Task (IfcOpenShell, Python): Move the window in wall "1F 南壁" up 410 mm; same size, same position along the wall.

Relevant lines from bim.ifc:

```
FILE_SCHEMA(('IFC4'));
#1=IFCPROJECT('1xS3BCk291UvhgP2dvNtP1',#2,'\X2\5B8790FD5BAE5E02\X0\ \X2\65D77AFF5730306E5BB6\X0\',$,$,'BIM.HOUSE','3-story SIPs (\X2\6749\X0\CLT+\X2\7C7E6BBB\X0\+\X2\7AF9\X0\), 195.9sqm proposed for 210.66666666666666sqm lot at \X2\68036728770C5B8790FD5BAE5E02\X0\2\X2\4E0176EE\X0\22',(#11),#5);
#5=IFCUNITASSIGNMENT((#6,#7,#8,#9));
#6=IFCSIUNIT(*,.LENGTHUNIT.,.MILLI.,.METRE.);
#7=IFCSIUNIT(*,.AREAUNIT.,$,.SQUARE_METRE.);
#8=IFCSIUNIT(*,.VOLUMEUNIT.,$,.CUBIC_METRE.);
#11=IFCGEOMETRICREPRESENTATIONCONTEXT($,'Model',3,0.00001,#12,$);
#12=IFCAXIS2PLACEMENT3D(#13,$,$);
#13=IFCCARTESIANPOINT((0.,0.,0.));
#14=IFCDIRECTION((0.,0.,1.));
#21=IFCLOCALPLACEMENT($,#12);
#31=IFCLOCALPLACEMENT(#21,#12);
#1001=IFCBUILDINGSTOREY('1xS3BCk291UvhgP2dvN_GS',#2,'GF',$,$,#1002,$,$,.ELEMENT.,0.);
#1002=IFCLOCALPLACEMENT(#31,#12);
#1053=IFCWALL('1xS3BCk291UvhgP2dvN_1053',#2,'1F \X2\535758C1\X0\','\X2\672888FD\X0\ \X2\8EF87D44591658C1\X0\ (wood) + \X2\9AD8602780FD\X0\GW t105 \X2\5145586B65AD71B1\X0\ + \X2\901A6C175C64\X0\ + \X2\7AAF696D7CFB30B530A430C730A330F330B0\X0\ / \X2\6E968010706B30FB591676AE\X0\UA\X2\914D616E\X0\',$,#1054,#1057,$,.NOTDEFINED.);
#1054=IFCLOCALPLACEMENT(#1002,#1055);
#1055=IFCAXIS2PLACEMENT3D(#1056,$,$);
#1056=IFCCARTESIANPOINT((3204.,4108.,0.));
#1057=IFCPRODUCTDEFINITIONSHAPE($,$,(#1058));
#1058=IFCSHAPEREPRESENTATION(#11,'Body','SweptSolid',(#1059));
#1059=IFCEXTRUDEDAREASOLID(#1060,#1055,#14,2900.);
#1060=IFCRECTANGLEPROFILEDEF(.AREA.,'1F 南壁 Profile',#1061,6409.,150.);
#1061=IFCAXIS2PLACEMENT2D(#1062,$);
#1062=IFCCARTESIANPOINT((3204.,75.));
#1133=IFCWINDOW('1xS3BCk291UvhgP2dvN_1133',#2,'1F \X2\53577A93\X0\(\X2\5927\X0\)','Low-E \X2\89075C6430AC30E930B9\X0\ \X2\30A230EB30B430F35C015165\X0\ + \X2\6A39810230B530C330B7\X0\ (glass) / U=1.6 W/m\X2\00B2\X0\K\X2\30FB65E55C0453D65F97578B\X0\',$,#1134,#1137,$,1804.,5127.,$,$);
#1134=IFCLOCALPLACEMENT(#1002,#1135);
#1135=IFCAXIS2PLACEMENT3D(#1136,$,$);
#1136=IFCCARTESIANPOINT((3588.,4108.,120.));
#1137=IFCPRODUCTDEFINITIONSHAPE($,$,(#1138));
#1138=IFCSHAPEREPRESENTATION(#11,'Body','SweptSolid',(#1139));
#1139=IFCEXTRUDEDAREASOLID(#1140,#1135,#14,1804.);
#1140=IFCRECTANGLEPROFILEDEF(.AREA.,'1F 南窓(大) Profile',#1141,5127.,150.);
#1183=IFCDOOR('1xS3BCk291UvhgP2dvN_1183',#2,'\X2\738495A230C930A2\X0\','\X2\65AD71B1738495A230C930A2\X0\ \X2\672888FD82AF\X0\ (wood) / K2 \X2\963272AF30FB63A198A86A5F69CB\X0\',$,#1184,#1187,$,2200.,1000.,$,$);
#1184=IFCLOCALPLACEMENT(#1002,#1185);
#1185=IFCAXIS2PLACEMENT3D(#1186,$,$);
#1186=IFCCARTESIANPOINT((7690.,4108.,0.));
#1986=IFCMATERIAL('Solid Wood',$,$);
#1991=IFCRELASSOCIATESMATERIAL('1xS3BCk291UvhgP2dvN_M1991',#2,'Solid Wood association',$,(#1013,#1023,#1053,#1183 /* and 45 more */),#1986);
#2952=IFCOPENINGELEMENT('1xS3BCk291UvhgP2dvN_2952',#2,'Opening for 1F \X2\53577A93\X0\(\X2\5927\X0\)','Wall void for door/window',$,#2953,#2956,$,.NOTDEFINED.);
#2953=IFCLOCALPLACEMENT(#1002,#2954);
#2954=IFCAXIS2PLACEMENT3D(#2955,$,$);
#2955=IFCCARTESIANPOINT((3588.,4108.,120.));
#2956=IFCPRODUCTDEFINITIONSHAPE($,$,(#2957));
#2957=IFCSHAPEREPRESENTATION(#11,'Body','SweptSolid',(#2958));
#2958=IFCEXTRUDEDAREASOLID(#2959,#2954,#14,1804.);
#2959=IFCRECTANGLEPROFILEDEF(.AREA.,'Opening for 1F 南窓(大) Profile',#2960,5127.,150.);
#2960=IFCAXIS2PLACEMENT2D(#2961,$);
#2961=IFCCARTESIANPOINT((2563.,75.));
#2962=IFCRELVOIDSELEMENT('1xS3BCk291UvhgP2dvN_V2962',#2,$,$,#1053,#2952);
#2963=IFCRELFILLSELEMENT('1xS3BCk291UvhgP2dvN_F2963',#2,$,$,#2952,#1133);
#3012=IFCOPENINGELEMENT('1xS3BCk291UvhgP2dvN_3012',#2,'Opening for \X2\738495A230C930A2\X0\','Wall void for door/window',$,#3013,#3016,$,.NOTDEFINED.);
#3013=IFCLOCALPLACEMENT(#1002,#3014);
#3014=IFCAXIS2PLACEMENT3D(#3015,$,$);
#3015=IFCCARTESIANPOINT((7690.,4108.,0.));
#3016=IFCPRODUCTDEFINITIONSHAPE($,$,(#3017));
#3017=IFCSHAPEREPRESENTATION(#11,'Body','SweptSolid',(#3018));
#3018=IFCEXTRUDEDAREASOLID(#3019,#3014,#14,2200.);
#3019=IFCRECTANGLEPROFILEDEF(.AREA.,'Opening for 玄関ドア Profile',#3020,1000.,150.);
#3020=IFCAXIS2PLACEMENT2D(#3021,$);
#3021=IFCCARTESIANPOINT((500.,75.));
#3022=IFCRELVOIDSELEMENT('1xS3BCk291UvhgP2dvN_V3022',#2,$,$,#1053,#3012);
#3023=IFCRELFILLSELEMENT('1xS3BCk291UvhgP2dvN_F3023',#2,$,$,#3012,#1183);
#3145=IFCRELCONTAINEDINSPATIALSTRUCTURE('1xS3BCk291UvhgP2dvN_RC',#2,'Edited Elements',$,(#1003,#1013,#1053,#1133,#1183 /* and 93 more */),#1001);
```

```python
import numpy as np
import ifcopenshell
import ifcopenshell.api.geometry
import ifcopenshell.util.placement
import ifcopenshell.util.unit

model = ifcopenshell.open("bim.ifc")
unit_scale = ifcopenshell.util.unit.calculate_unit_scale(model)

window = model.by_guid("1xS3BCk291UvhgP2dvN_1133")
opening = window.FillsVoids[0].RelatingOpeningElement
dz = 0.41 / unit_scale

shift = np.array([0.0, 0.0, dz])
# The window is not placed relative to its opening, so move both.
for product in (opening, window):
    matrix = ifcopenshell.util.placement.get_local_placement(product.ObjectPlacement)
    matrix[:3, 3] += shift
    ifcopenshell.api.geometry.edit_object_placement(model, product=product, matrix=matrix, is_si=False)

print(f"moved by {dz * unit_scale:+.3f} m")

model.write("bim_v2.ifc")
```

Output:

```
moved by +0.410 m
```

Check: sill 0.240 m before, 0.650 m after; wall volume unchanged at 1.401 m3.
